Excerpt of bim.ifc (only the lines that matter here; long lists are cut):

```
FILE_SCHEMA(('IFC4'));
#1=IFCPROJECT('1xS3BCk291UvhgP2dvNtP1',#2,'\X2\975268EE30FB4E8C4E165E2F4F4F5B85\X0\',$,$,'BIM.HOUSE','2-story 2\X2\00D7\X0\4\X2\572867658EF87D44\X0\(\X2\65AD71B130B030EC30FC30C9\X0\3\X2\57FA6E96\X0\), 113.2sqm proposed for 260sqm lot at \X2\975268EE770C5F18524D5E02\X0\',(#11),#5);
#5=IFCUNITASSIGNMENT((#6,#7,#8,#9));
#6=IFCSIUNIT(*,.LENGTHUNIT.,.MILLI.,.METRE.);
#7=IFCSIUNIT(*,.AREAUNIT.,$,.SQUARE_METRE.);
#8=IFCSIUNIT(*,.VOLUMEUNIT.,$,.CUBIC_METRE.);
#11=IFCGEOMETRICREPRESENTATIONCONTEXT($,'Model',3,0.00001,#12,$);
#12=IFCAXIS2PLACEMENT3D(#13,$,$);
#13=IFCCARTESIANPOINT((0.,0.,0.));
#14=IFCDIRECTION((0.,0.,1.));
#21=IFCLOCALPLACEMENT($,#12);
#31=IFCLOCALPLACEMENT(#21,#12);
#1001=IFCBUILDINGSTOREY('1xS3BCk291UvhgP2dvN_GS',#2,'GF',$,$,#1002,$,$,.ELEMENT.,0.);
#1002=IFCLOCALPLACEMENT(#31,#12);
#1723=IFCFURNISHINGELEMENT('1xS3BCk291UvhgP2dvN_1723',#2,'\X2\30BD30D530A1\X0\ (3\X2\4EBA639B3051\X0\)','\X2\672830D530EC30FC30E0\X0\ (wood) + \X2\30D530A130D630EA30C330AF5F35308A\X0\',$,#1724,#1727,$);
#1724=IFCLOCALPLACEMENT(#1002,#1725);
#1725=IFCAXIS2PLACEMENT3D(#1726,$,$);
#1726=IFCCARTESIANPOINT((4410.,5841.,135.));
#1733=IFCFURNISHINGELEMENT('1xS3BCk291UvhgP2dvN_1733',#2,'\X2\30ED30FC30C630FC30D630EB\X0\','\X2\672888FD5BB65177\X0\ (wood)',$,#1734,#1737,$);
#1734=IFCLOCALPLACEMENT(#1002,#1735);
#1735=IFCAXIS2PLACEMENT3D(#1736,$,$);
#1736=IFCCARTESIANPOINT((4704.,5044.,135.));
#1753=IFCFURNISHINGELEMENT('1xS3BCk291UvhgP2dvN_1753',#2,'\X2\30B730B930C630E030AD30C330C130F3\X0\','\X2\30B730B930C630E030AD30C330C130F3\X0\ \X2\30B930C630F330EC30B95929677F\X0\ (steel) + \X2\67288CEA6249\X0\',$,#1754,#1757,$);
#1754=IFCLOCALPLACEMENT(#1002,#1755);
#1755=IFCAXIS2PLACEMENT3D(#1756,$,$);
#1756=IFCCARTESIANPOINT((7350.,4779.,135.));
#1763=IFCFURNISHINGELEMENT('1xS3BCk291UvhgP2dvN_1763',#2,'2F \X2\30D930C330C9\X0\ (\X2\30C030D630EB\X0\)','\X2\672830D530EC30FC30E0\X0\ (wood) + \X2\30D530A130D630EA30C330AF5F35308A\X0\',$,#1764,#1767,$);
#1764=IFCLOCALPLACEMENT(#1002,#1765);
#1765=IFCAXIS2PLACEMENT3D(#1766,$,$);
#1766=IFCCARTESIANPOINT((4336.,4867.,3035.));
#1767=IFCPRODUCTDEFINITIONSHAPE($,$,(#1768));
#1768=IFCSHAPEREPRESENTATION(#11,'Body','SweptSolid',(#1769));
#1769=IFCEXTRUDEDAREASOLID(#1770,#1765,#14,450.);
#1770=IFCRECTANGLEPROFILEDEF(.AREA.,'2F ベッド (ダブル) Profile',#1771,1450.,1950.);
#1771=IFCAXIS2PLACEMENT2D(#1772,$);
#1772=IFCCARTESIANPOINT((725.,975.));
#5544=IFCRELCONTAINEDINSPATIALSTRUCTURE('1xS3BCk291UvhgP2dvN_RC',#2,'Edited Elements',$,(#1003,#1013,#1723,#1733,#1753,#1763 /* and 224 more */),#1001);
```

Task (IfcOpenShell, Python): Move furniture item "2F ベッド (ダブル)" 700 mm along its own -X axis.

```python
import ifcopenshell
import ifcopenshell.api.geometry
import ifcopenshell.util.placement

model = ifcopenshell.open("bim.ifc")

item = model.by_id(1763)
matrix = ifcopenshell.util.placement.get_local_placement(item.ObjectPlacement)
matrix[:3, 3] -= matrix[:3, 0] * 700.0
ifcopenshell.api.geometry.edit_object_placement(model, product=item, matrix=matrix, is_si=False)

print(ifcopenshell.util.placement.get_local_placement(item.ObjectPlacement).round(3) + 0.0)

model.write("bim_rev.ifc")
```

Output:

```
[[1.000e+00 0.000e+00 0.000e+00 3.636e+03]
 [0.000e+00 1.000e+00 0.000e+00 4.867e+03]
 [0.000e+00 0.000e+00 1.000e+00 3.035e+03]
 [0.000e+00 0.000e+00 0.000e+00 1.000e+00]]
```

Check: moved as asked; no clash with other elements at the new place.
